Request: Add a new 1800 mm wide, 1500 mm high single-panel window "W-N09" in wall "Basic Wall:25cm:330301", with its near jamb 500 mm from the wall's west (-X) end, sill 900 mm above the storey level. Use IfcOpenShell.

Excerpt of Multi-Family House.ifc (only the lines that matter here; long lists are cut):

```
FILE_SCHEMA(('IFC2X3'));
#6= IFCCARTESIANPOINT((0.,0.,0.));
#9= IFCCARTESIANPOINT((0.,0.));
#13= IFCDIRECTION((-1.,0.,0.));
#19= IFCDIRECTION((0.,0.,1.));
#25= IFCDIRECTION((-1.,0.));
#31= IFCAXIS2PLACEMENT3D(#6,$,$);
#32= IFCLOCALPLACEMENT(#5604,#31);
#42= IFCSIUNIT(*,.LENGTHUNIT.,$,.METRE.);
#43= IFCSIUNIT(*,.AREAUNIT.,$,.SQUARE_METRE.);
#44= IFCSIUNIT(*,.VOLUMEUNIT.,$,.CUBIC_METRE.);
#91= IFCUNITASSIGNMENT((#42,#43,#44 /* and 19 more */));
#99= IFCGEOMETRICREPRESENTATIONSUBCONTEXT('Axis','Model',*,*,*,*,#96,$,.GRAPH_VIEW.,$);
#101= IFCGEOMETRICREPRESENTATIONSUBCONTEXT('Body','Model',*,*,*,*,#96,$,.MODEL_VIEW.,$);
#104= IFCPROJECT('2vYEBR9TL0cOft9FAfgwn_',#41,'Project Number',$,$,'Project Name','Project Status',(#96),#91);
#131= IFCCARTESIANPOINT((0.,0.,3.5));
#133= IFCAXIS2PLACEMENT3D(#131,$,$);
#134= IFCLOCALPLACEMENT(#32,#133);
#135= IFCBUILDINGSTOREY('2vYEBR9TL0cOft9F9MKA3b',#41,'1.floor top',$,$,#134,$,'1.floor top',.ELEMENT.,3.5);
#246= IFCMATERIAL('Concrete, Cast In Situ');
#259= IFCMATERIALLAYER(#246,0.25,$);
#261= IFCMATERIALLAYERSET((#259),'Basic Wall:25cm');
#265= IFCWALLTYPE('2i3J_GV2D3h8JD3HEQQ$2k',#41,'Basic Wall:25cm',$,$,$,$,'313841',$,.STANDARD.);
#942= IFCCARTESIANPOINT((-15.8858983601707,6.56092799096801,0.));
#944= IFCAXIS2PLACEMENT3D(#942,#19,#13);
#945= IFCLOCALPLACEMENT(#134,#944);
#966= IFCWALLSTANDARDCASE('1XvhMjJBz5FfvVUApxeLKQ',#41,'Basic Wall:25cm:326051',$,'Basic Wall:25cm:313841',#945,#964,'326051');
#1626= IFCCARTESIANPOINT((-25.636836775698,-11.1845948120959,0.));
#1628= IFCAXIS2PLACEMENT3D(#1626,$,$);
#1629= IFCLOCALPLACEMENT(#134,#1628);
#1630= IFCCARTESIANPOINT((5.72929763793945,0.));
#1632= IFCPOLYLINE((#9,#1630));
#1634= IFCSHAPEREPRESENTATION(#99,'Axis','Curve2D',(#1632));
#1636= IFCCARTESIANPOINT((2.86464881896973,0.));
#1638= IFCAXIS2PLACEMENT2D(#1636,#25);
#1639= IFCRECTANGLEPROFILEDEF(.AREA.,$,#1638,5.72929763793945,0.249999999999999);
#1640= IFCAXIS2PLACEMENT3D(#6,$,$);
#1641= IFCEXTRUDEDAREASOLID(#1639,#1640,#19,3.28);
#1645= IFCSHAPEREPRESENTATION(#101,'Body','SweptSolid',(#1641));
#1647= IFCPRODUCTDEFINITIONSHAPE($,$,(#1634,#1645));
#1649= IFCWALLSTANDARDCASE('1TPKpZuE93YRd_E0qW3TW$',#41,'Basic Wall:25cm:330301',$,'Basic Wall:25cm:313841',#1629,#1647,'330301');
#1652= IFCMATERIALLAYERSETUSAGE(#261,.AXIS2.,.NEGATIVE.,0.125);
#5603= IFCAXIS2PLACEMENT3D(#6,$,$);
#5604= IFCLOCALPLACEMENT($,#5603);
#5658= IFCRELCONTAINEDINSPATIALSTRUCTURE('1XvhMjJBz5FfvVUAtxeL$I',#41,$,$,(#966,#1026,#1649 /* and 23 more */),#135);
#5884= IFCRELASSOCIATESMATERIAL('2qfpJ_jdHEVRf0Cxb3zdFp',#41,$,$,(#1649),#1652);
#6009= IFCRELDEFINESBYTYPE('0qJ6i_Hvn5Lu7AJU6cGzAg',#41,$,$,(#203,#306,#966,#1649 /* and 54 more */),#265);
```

```python
import numpy as np
import ifcopenshell
import ifcopenshell.api.feature
import ifcopenshell.api.geometry
import ifcopenshell.api.root
import ifcopenshell.api.spatial
import ifcopenshell.api.type
import ifcopenshell.geom
import ifcopenshell.util.element
import ifcopenshell.util.placement
import ifcopenshell.util.representation
import ifcopenshell.util.shape
import ifcopenshell.util.unit

model = ifcopenshell.open("Multi-Family House.ifc")
unit_scale = ifcopenshell.util.unit.calculate_unit_scale(model)
settings = ifcopenshell.geom.settings()


def volume(element):
    """Net volume in cubic metres, openings subtracted."""
    shape = ifcopenshell.geom.create_shape(settings, element)
    return ifcopenshell.util.shape.get_volume(shape.geometry)


wall = model.by_guid("1TPKpZuE93YRd_E0qW3TW$")
storey = ifcopenshell.util.element.get_container(wall, ifc_class="IfcBuildingStorey")
context = ifcopenshell.util.representation.get_context(model, "Model", "Body", "MODEL_VIEW")
before = volume(wall)

width, height, from_end, sill = 1.8, 1.5, 0.5, 0.9  # metres

# The wall runs along its own X axis, and the end named is its -X end.
wall_shape = ifcopenshell.geom.create_shape(settings, wall)
x, y, z = ifcopenshell.util.shape.get_vertices(wall_shape.geometry).T
start = x.min() + from_end
face, thickness = float(y.min()), float(y.max() - y.min())
wall_matrix = ifcopenshell.util.placement.get_local_placement(wall.ObjectPlacement)
level = ifcopenshell.util.placement.get_local_placement(storey.ObjectPlacement)[2, 3]


def in_wall(x, y):
    """Placement at x, y metres in the wall's axes, at sill height."""
    matrix = wall_matrix.copy()
    matrix[:, 3] = wall_matrix @ np.array([x / unit_scale, y / unit_scale, 0.0, 1.0])
    matrix[2, 3] = level + sill / unit_scale
    return matrix


# Opening: a box that overshoots both wall faces by 50 mm.
opening = ifcopenshell.api.root.create_entity(model, ifc_class="IfcOpeningElement")
box = ifcopenshell.api.geometry.add_wall_representation(
    model, context=context, length=width, height=height, thickness=thickness + 0.1
)
ifcopenshell.api.geometry.assign_representation(model, product=opening, representation=box)
ifcopenshell.api.geometry.edit_object_placement(model, product=opening, matrix=in_wall(start, face - 0.05), is_si=False)
ifcopenshell.api.feature.add_feature(model, feature=opening, element=wall)

window = ifcopenshell.api.root.create_entity(model, ifc_class="IfcWindow", name="W-N09")
window.OverallWidth, window.OverallHeight = width / unit_scale, height / unit_scale
body = ifcopenshell.api.geometry.add_window_representation(
    model,
    context=context,
    overall_width=window.OverallWidth,
    overall_height=window.OverallHeight,
    partition_type="SINGLE_PANEL",
)
ifcopenshell.api.geometry.assign_representation(model, product=window, representation=body)
ifcopenshell.api.spatial.assign_container(model, products=[window], relating_structure=storey)
fills = ifcopenshell.api.feature.add_filling(model, opening=opening, element=window)
fills.OwnerHistory = window.OwnerHistory  # required in IFC2X3

# IFC2X3 keeps the operation on the window style.
style = ifcopenshell.api.root.create_entity(model, ifc_class="IfcWindowStyle", name="W-N09")
style.OperationType, style.ConstructionType = "SINGLE_PANEL", "NOTDEFINED"
style.ParameterTakesPrecedence = style.Sizeable = False
ifcopenshell.api.type.assign_type(model, related_objects=[window], relating_type=style)

# Centre the window in the wall's thickness.
ifcopenshell.api.geometry.edit_object_placement(model, product=window, matrix=in_wall(start, face), is_si=False)
window_shape = ifcopenshell.geom.create_shape(settings, window)
depth = ifcopenshell.util.shape.get_vertices(window_shape.geometry)[:, 1]
offset = face + thickness / 2 - (depth.min() + depth.max()) / 2
ifcopenshell.api.geometry.edit_object_placement(model, product=window, matrix=in_wall(start, offset), is_si=False)

after = volume(wall)

print(f"wall volume {before:.3f} -> {after:.3f} m3")

model.write("Multi-Family House_rev.ifc")
```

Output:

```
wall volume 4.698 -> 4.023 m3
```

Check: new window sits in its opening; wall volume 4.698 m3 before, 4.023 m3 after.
